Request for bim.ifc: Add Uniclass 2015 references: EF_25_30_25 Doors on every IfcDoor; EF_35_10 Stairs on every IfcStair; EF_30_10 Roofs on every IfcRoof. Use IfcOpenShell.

First a look at what the model holds.

```python
import ifcopenshell

model = ifcopenshell.open("bim.ifc")
print(model.schema)
print("classifications:", [c.Name for c in model.by_type("IfcClassification")])
for ifc_class in ("IfcDoor", "IfcRoof", "IfcStair", "IfcWall", "IfcWindow"):
    print(ifc_class, len(model.by_type(ifc_class)))
```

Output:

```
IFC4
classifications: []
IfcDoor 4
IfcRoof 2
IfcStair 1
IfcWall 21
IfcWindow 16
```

```python
import ifcopenshell
import ifcopenshell.api.classification

model = ifcopenshell.open("bim.ifc")

system = ifcopenshell.api.classification.add_classification(model, classification="Uniclass 2015")

codes = {
    "IfcDoor": ("EF_25_30_25", "Doors"),
    "IfcStair": ("EF_35_10", "Stairs"),
    "IfcRoof": ("EF_30_10", "Roofs"),
}
for ifc_class, (code, name) in codes.items():
    products = model.by_type(ifc_class)
    ifcopenshell.api.classification.add_reference(
        model, products=products, classification=system, identification=code, name=name
    )
    print(code, len(products))

model.write("bim_edited.ifc")
```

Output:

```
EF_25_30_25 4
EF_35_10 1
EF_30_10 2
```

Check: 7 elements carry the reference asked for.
